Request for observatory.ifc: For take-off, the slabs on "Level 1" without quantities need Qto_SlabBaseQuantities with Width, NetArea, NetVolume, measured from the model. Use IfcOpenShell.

First a look at what the model holds.

```python
import ifcopenshell
import ifcopenshell.util.element
import ifcopenshell.util.unit

model = ifcopenshell.open("observatory.ifc")
print(model.schema)
for unit_type in ("LENGTHUNIT", "AREAUNIT", "VOLUMEUNIT"):
    print(unit_type, ifcopenshell.util.unit.calculate_unit_scale(model, unit_type))
storey = next(s for s in model.by_type("IfcBuildingStorey") if s.Name == "Level 1")
slabs = [e for e in ifcopenshell.util.element.get_decomposition(storey) if e.is_a("IfcSlab")]
for e in sorted(slabs, key=lambda e: e.id()):
    print(e.id(), e.is_a(), e.Name, list(ifcopenshell.util.element.get_psets(e, qtos_only=True)), sep=" | ")
```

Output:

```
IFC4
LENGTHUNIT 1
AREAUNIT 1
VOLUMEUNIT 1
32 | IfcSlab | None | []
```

```python
import ifcopenshell
import ifcopenshell.api.pset
import ifcopenshell.geom
import ifcopenshell.util.element
import ifcopenshell.util.shape
import ifcopenshell.util.unit

model = ifcopenshell.open("observatory.ifc")
unit_scale = ifcopenshell.util.unit.calculate_unit_scale(model)
area_scale = ifcopenshell.util.unit.calculate_unit_scale(model, "AREAUNIT")
volume_scale = ifcopenshell.util.unit.calculate_unit_scale(model, "VOLUMEUNIT")
settings = ifcopenshell.geom.settings()

storey = next(s for s in model.by_type("IfcBuildingStorey") if s.Name == "Level 1")
slabs = [e for e in ifcopenshell.util.element.get_decomposition(storey) if e.is_a("IfcSlab")]

for e in sorted(slabs, key=lambda e: e.id()):
    if ifcopenshell.util.element.get_psets(e, qtos_only=True, should_inherit=False):
        continue
    # Geometry comes back in metres, in the element's own axes.
    shape = ifcopenshell.geom.create_shape(settings, e)
    values = {
        "Width": ifcopenshell.util.shape.get_z(shape.geometry) / unit_scale,
        "NetArea": ifcopenshell.util.shape.get_footprint_area(shape.geometry) / area_scale,
        "NetVolume": ifcopenshell.util.shape.get_volume(shape.geometry) / volume_scale,
    }
    qto = ifcopenshell.api.pset.add_qto(model, product=e, name="Qto_SlabBaseQuantities")
    ifcopenshell.api.pset.edit_qto(model, qto=qto, properties=values)
    print(e.id(), {k: round(v, 3) for k, v in values.items()})

model.write("observatory-out.ifc")
```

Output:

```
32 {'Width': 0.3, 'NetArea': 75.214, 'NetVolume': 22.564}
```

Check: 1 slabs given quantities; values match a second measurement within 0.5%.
